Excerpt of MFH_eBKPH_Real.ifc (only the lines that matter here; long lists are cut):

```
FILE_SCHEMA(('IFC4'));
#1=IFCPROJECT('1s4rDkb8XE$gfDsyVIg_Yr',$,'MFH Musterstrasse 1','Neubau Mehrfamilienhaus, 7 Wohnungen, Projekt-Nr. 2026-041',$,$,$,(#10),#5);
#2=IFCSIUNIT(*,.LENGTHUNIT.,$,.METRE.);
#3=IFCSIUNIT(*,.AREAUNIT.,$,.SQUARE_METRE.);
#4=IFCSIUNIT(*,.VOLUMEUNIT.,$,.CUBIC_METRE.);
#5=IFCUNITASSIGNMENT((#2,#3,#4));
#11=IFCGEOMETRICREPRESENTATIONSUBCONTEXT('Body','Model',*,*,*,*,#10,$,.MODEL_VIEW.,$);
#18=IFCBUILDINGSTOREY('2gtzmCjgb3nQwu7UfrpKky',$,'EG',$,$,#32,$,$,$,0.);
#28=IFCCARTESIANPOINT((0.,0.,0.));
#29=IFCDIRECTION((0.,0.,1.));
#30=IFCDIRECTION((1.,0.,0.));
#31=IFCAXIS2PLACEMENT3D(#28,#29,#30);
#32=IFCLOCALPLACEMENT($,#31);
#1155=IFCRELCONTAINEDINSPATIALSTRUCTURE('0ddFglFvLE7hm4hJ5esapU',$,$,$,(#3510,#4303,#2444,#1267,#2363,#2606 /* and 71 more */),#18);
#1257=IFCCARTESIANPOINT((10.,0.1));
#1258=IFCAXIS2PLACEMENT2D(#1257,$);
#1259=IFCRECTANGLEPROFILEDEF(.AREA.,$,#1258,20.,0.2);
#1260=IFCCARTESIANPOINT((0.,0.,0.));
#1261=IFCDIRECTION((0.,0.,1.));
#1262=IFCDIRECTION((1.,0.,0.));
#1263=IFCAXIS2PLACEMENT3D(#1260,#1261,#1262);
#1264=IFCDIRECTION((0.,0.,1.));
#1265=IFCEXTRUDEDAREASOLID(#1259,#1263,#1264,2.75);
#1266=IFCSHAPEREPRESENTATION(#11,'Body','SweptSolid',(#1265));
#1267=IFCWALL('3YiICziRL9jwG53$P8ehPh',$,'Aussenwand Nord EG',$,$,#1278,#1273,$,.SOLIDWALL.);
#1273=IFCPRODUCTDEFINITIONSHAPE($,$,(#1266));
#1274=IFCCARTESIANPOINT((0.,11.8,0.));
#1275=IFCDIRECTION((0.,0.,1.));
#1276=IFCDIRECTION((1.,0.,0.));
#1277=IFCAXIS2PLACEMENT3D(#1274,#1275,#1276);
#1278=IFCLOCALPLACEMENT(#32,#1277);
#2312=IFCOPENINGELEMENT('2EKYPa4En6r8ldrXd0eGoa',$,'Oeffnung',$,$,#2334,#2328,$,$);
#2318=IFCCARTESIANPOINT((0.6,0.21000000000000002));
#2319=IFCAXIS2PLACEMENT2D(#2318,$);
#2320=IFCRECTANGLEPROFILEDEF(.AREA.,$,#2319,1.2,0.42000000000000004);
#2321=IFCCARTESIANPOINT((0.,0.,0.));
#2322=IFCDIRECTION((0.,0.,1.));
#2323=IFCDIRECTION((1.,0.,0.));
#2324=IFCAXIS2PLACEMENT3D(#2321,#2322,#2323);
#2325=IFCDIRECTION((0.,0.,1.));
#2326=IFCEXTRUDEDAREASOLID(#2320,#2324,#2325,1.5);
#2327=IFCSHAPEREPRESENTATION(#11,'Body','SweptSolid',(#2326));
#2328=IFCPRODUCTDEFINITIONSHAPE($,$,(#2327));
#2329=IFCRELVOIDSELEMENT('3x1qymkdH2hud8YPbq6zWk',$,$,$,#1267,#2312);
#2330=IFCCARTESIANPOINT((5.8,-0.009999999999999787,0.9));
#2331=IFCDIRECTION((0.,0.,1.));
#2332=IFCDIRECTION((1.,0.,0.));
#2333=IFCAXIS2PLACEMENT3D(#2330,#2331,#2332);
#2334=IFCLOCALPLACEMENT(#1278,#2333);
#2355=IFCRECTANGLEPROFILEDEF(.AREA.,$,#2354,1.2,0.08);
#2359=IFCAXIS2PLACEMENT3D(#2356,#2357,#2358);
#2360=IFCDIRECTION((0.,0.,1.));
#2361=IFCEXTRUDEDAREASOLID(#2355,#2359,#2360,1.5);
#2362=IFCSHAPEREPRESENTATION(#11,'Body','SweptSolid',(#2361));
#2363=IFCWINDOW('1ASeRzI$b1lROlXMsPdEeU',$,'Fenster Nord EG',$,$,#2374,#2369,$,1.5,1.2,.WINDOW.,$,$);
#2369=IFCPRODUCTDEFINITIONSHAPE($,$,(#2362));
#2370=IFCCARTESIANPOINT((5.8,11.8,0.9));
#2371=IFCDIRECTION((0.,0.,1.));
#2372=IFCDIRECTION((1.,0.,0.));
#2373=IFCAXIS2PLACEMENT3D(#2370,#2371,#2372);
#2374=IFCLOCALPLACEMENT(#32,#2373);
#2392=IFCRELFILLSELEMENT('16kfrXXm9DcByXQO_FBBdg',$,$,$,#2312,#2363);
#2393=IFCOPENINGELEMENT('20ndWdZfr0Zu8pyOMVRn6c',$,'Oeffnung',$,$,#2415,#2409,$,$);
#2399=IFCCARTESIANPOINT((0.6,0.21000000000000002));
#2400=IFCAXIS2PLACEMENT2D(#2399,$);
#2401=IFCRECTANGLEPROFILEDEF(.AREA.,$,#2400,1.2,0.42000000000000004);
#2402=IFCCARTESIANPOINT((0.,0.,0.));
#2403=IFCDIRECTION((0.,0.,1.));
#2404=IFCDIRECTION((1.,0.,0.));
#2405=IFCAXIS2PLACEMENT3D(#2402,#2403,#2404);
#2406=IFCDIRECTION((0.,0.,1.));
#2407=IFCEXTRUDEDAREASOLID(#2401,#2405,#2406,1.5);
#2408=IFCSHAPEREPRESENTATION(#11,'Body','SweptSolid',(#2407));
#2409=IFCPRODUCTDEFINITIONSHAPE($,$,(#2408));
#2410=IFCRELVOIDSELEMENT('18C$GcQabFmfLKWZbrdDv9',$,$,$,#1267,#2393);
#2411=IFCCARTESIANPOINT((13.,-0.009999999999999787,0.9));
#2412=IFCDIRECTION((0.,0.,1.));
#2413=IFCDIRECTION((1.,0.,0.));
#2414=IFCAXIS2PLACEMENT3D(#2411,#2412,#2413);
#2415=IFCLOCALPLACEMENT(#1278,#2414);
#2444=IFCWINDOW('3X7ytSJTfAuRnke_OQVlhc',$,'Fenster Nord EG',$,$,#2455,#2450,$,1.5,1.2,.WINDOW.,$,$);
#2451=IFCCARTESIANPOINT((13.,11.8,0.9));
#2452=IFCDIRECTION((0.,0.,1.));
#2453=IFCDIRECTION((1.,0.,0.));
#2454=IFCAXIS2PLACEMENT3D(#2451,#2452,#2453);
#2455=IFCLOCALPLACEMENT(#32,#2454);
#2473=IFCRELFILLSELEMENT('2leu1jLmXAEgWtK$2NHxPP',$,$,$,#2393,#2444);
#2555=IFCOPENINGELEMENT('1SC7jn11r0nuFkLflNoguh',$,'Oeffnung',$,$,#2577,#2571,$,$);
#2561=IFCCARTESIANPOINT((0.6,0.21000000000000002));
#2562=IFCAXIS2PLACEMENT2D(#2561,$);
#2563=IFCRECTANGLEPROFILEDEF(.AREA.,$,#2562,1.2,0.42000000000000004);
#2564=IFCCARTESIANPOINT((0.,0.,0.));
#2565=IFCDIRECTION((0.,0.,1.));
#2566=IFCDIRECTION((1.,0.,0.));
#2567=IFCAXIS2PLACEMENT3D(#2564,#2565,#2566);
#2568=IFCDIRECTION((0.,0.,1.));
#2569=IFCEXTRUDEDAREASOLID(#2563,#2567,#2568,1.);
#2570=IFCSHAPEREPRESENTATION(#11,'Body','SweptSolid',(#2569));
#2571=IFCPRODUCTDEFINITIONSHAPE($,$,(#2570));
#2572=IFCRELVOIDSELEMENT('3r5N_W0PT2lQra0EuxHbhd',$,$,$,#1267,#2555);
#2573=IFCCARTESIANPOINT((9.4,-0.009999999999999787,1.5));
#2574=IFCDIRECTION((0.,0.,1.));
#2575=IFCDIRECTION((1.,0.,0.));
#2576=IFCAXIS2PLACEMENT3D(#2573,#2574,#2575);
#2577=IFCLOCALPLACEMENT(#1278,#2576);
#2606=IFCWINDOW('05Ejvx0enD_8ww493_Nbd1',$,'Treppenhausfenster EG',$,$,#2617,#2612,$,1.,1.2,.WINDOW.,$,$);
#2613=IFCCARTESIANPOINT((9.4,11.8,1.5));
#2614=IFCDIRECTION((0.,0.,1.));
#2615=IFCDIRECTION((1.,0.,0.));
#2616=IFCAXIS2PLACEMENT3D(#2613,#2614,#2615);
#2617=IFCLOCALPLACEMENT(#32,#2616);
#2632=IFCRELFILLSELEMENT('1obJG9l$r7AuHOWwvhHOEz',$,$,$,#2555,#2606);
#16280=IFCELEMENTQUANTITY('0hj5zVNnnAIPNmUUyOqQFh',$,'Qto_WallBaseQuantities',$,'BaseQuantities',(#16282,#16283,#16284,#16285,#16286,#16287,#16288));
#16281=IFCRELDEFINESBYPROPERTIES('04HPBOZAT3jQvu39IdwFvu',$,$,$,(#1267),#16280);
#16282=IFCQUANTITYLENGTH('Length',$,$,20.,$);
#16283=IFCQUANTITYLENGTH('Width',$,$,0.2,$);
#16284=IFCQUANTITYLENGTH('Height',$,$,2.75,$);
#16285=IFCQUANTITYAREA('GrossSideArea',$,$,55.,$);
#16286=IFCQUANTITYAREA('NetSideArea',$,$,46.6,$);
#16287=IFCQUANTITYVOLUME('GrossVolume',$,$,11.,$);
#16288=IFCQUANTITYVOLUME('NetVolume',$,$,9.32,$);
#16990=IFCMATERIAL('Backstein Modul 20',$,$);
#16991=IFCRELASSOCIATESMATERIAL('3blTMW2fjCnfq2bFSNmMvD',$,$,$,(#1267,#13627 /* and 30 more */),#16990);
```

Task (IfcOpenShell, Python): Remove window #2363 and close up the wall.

```python
import ifcopenshell
import ifcopenshell.api.feature
import ifcopenshell.api.pset
import ifcopenshell.api.root
import ifcopenshell.geom
import ifcopenshell.util.element
import ifcopenshell.util.shape
import ifcopenshell.util.unit

model = ifcopenshell.open("MFH_eBKPH_Real.ifc")
area_scale = ifcopenshell.util.unit.calculate_unit_scale(model, "AREAUNIT")
volume_scale = ifcopenshell.util.unit.calculate_unit_scale(model, "VOLUMEUNIT")
settings = ifcopenshell.geom.settings()


def volume(element):
    """Net volume in cubic metres, openings subtracted."""
    shape = ifcopenshell.geom.create_shape(settings, element)
    return ifcopenshell.util.shape.get_volume(shape.geometry)


window = model.by_id(2363)
opening = window.FillsVoids[0].RelatingOpeningElement
wall = opening.VoidsElements[0].RelatingBuildingElement
before = volume(wall)

ifcopenshell.api.root.remove_product(model, product=window)
ifcopenshell.api.feature.remove_feature(model, feature=opening)

after = volume(wall)
thickness = 0.2  # wall thickness in metres

# Update the wall's stored quantities.
qto = model.by_id(ifcopenshell.util.element.get_pset(wall, "Qto_WallBaseQuantities", should_inherit=False)["id"])
ifcopenshell.api.pset.edit_qto(model, qto=qto, properties={
    "NetSideArea": after / thickness / area_scale,
    "NetVolume": after / volume_scale,
})

print(f"wall volume {before:.3f} -> {after:.3f} m3")

model.write("MFH_eBKPH_Real_v2.ifc")
```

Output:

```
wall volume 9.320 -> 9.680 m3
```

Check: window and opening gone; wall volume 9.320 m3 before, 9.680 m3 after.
